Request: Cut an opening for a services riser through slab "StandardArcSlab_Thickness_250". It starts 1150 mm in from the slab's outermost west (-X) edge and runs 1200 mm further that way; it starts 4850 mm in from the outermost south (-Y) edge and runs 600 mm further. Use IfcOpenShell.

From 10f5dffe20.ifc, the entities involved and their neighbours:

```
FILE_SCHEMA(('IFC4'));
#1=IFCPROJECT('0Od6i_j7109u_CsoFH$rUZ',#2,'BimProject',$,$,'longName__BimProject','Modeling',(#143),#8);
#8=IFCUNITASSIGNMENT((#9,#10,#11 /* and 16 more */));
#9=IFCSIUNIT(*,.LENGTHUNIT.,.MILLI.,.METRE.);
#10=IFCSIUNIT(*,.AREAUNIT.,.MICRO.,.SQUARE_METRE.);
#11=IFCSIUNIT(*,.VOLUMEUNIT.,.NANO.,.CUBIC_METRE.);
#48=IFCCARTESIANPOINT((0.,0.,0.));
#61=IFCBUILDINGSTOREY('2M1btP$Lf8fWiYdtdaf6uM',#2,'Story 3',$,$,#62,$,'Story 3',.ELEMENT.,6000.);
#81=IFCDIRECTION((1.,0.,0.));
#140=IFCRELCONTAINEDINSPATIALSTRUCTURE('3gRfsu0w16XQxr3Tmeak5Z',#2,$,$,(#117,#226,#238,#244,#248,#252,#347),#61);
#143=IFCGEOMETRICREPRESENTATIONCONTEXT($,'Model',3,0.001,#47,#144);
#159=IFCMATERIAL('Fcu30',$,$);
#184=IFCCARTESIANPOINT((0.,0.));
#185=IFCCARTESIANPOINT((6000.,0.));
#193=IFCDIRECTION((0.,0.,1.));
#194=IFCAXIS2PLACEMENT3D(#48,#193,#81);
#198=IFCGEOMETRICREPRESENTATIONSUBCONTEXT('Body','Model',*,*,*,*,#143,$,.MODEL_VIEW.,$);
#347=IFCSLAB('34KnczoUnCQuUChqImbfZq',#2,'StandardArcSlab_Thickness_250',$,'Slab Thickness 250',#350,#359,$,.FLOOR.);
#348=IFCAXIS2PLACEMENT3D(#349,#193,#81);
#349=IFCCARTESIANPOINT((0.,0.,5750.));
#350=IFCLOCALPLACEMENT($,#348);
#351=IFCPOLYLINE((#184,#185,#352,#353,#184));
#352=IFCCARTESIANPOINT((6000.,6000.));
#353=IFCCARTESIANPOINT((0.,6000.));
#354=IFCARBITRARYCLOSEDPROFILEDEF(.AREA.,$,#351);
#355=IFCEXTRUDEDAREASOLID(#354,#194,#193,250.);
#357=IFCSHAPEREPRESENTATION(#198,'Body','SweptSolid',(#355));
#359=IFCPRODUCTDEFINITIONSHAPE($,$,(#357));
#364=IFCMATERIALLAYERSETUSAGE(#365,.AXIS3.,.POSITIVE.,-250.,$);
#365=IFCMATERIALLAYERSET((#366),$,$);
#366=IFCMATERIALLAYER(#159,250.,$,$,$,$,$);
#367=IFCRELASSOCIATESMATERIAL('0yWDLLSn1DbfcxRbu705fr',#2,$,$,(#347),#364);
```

```python
import numpy as np
import ifcopenshell
import ifcopenshell.api.feature
import ifcopenshell.api.geometry
import ifcopenshell.api.root
import ifcopenshell.geom
import ifcopenshell.util.placement
import ifcopenshell.util.representation
import ifcopenshell.util.shape
import ifcopenshell.util.unit

model = ifcopenshell.open("10f5dffe20.ifc")
unit_scale = ifcopenshell.util.unit.calculate_unit_scale(model)
settings = ifcopenshell.geom.settings()


def volume(element):
    """Net volume in cubic metres, openings subtracted."""
    shape = ifcopenshell.geom.create_shape(settings, element)
    return ifcopenshell.util.shape.get_volume(shape.geometry)


slab = model.by_guid("34KnczoUnCQuUChqImbfZq")
before = volume(slab)

# Extent in the slab's own axes, in metres. The edges named are its -X and -Y sides.
slab_shape = ifcopenshell.geom.create_shape(settings, slab)
vertices = ifcopenshell.util.shape.get_vertices(slab_shape.geometry)
x_min, y_min, bottom = vertices.min(axis=0)
top = vertices[:, 2].max()

opening = ifcopenshell.api.root.create_entity(model, ifc_class="IfcOpeningElement", name="Services riser opening", predefined_type="OPENING")
context = ifcopenshell.util.representation.get_context(model, "Model", "Body", "MODEL_VIEW")
width, depth = 1.2, 0.6
outline = [(0.0, 0.0), (width, 0.0), (width, depth), (0.0, depth), (0.0, 0.0)]
# Overshoot both faces by 50 mm so the cut is clean.
shape = ifcopenshell.api.geometry.add_slab_representation(
    model, context=context, depth=top - bottom + 0.1, polyline=outline
)
ifcopenshell.api.geometry.assign_representation(model, product=opening, representation=shape)

matrix = ifcopenshell.util.placement.get_local_placement(slab.ObjectPlacement)
matrix[:, 3] = matrix @ np.append(np.array([x_min + 1.15, y_min + 4.85, bottom - 0.05]) / unit_scale, 1.0)
ifcopenshell.api.geometry.edit_object_placement(model, product=opening, matrix=matrix, is_si=False)
ifcopenshell.api.feature.add_feature(model, feature=opening, element=slab)

after = volume(slab)

print(f"slab volume {before:.3f} -> {after:.3f} m3")

model.write("10f5dffe20_v2.ifc")
```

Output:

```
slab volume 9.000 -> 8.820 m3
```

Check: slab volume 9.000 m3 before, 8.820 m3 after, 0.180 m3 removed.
